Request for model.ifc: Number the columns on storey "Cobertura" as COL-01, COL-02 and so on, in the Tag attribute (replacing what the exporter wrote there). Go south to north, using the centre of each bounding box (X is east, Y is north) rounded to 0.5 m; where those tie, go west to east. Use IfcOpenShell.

First a look at what the model holds.

```python
import ifcopenshell
import ifcopenshell.util.element
import ifcopenshell.util.placement

model = ifcopenshell.open("model.ifc")
print(model.schema)
storey = next(s for s in model.by_type("IfcBuildingStorey") if s.Name == "Cobertura")
columns = [e for e in ifcopenshell.util.element.get_decomposition(storey) if e.is_a("IfcColumn")]
for e in sorted(columns, key=lambda e: e.id()):
    origin = ifcopenshell.util.placement.get_local_placement(e.ObjectPlacement)[:3, 3]
    print(e.id(), e.Tag, e.Name, origin.round(2) + 0.0, sep=" | ")
```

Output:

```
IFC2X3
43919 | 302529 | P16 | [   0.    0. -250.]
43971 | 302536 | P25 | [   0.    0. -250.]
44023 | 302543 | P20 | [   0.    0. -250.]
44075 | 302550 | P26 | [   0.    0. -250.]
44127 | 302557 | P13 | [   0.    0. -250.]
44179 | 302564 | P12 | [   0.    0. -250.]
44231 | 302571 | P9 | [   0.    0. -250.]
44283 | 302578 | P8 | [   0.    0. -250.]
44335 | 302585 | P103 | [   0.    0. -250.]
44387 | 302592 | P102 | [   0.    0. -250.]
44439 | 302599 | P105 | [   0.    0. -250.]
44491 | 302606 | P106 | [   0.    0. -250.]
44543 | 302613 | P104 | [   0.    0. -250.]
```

```python
import ifcopenshell
import ifcopenshell.geom
import ifcopenshell.util.element
import ifcopenshell.util.shape

model = ifcopenshell.open("model.ifc")
settings = ifcopenshell.geom.settings()
settings.set("use-world-coords", True)


def centre(element):
    shape = ifcopenshell.geom.create_shape(settings, element)
    return ifcopenshell.util.shape.get_bbox_centroid(shape.geometry)


storey = next(s for s in model.by_type("IfcBuildingStorey") if s.Name == "Cobertura")
columns = [e for e in ifcopenshell.util.element.get_decomposition(storey) if e.is_a("IfcColumn")]

# Insertion points can sit at a corner or the storey origin, so sort by the geometry (in metres).
centres = {e: centre(e) for e in columns}
columns.sort(key=lambda e: (round(centres[e][1] / 0.5), centres[e][0]))

for i, e in enumerate(columns, start=1):
    number = f"COL-{i:02d}"
    e.Tag = number
    print(e.id(), number)

model.write("model_updated.ifc")
```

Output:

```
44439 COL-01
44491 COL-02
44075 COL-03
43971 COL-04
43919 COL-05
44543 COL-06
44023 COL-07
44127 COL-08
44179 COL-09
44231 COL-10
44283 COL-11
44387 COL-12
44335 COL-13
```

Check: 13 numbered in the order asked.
